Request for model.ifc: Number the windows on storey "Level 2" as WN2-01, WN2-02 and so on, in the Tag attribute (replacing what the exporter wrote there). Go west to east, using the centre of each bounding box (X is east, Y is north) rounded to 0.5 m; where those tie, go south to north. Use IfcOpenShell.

First a look at what the model holds.

```python
import ifcopenshell
import ifcopenshell.util.element
import ifcopenshell.util.placement

model = ifcopenshell.open("model.ifc")
print(model.schema)
storey = next(s for s in model.by_type("IfcBuildingStorey") if s.Name == "Level 2")
windows = [e for e in ifcopenshell.util.element.get_decomposition(storey) if e.is_a("IfcWindow")]
for e in sorted(windows, key=lambda e: e.id()):
    origin = ifcopenshell.util.placement.get_local_placement(e.ObjectPlacement)[:3, 3]
    print(e.id(), e.Tag, e.Name, origin.round(2) + 0.0, sep=" | ")
```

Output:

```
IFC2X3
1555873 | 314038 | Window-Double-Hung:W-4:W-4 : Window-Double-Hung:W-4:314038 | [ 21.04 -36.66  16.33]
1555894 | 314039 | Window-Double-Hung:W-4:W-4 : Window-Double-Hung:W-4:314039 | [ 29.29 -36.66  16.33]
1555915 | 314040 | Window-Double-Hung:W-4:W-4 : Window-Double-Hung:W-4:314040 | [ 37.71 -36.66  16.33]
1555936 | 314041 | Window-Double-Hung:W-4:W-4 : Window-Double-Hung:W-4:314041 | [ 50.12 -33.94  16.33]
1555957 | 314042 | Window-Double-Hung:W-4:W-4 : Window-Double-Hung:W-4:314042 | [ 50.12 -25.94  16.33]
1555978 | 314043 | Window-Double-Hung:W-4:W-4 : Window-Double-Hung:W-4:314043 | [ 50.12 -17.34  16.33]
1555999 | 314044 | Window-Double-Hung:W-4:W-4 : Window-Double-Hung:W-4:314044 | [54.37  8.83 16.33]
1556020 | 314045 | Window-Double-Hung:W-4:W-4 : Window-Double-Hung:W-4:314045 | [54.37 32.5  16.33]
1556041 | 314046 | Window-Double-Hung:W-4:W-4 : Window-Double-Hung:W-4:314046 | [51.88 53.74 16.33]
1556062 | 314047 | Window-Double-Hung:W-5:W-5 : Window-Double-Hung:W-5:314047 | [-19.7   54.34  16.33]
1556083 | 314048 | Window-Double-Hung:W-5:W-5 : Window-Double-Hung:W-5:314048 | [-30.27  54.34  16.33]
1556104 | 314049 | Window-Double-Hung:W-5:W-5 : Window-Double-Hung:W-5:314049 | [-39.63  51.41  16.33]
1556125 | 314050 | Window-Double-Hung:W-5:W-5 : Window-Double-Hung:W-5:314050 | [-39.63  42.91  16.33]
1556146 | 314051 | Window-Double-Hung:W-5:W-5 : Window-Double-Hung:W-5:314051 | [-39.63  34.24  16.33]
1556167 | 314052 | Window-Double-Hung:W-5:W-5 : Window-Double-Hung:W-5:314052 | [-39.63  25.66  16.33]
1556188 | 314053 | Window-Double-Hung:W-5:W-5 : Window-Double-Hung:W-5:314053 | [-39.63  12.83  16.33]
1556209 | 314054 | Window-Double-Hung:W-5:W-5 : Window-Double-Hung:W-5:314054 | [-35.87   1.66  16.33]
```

```python
import ifcopenshell
import ifcopenshell.geom
import ifcopenshell.util.element
import ifcopenshell.util.shape

model = ifcopenshell.open("model.ifc")
settings = ifcopenshell.geom.settings()
settings.set("use-world-coords", True)


def centre(element):
    shape = ifcopenshell.geom.create_shape(settings, element)
    return ifcopenshell.util.shape.get_bbox_centroid(shape.geometry)


storey = next(s for s in model.by_type("IfcBuildingStorey") if s.Name == "Level 2")
windows = [e for e in ifcopenshell.util.element.get_decomposition(storey) if e.is_a("IfcWindow")]

# Insertion points can sit at a corner or the storey origin, so sort by the geometry (in metres).
centres = {e: centre(e) for e in windows}
windows.sort(key=lambda e: (round(centres[e][0] / 0.5), centres[e][1]))

for i, e in enumerate(windows, start=1):
    number = f"WN2-{i:02d}"
    e.Tag = number
    print(e.id(), number)

model.write("model_v2.ifc")
```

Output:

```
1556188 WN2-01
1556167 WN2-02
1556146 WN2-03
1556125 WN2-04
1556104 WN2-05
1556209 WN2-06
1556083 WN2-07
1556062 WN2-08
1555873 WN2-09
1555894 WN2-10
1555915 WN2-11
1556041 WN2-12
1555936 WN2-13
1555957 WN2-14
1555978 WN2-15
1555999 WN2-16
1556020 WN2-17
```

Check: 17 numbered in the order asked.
